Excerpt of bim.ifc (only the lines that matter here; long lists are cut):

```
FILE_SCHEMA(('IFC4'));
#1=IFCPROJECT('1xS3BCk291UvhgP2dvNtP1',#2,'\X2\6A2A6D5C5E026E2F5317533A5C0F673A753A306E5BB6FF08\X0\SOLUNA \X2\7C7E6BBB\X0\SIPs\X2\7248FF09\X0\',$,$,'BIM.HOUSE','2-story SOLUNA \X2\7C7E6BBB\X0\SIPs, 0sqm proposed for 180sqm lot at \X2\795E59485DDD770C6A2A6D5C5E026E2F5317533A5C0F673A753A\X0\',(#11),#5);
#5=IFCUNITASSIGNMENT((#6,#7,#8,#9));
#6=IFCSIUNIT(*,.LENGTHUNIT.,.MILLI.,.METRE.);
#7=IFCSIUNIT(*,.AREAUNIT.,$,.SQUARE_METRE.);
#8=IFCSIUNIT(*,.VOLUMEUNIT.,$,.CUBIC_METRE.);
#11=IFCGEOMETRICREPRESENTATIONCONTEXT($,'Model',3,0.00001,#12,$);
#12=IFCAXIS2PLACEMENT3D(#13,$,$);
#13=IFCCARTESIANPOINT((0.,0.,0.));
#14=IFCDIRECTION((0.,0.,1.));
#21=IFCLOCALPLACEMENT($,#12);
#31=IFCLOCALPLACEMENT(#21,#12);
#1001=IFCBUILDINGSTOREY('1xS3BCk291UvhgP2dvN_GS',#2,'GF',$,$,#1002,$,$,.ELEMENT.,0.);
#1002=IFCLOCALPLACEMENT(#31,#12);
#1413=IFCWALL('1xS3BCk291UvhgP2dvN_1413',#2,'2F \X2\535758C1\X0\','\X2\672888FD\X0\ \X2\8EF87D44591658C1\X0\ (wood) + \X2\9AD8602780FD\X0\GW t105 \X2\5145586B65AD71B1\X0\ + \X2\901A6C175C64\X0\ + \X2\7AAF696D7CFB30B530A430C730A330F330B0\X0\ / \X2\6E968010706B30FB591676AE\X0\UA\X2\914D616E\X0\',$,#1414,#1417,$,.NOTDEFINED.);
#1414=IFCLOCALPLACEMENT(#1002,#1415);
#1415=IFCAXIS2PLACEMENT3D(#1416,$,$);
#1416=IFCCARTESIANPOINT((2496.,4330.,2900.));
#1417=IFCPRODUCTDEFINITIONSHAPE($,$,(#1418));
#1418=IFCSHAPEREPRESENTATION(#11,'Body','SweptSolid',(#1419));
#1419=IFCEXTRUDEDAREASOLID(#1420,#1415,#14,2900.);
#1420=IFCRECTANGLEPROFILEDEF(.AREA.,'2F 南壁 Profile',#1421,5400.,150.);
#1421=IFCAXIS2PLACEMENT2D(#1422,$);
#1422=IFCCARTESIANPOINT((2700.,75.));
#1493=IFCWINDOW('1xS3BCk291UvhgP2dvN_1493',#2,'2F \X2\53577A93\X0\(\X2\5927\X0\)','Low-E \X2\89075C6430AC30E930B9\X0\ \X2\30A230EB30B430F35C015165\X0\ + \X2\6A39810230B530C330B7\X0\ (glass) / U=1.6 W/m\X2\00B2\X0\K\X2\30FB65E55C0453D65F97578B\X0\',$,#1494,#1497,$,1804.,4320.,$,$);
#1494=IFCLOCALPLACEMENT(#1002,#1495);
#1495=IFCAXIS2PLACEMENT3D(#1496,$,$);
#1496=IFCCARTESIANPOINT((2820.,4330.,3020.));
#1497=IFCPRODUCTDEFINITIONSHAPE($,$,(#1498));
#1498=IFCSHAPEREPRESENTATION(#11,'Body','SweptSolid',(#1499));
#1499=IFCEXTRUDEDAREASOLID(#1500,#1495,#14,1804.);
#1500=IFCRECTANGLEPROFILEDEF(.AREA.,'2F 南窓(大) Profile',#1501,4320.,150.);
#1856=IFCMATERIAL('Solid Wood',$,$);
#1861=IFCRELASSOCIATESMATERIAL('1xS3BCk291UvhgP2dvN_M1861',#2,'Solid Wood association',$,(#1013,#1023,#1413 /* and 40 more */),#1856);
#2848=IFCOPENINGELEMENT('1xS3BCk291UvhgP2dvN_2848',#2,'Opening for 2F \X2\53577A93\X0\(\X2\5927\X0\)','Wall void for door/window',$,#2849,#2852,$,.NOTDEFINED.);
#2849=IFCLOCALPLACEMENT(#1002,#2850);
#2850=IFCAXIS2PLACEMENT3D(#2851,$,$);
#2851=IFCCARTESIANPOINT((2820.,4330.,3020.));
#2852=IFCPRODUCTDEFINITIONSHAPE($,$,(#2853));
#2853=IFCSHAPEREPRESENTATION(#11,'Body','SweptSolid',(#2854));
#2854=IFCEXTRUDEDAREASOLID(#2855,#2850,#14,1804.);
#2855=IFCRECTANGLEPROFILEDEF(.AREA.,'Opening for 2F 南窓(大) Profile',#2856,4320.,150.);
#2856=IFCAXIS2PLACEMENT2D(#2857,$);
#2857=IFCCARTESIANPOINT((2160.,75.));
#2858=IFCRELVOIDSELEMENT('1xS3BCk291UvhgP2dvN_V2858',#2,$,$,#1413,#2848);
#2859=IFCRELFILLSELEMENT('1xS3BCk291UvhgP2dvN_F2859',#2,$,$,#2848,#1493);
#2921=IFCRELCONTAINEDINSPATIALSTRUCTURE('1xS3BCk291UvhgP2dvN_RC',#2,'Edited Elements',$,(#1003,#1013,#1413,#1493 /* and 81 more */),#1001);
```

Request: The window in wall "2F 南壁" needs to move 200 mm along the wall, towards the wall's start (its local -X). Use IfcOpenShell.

```python
import ifcopenshell
import ifcopenshell.api.geometry
import ifcopenshell.util.placement
import ifcopenshell.util.unit

model = ifcopenshell.open("bim.ifc")
unit_scale = ifcopenshell.util.unit.calculate_unit_scale(model)

window = model.by_guid("1xS3BCk291UvhgP2dvN_1493")
opening = window.FillsVoids[0].RelatingOpeningElement
wall = opening.VoidsElements[0].RelatingBuildingElement

wall_matrix = ifcopenshell.util.placement.get_local_placement(wall.ObjectPlacement)
shift = wall_matrix[:3, 0] * -0.2 / unit_scale
before = ifcopenshell.util.placement.get_local_placement(window.ObjectPlacement)[:3, 3].copy()

# The window is not placed relative to its opening, so move both.
for product in (opening, window):
    matrix = ifcopenshell.util.placement.get_local_placement(product.ObjectPlacement)
    matrix[:3, 3] += shift
    ifcopenshell.api.geometry.edit_object_placement(model, product=product, matrix=matrix, is_si=False)

after = ifcopenshell.util.placement.get_local_placement(window.ObjectPlacement)[:3, 3]
print("window moved by", (after - before).round(3) + 0.0)

model.write("bim_updated.ifc")
```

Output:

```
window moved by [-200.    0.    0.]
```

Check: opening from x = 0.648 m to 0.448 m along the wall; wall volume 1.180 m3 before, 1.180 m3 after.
